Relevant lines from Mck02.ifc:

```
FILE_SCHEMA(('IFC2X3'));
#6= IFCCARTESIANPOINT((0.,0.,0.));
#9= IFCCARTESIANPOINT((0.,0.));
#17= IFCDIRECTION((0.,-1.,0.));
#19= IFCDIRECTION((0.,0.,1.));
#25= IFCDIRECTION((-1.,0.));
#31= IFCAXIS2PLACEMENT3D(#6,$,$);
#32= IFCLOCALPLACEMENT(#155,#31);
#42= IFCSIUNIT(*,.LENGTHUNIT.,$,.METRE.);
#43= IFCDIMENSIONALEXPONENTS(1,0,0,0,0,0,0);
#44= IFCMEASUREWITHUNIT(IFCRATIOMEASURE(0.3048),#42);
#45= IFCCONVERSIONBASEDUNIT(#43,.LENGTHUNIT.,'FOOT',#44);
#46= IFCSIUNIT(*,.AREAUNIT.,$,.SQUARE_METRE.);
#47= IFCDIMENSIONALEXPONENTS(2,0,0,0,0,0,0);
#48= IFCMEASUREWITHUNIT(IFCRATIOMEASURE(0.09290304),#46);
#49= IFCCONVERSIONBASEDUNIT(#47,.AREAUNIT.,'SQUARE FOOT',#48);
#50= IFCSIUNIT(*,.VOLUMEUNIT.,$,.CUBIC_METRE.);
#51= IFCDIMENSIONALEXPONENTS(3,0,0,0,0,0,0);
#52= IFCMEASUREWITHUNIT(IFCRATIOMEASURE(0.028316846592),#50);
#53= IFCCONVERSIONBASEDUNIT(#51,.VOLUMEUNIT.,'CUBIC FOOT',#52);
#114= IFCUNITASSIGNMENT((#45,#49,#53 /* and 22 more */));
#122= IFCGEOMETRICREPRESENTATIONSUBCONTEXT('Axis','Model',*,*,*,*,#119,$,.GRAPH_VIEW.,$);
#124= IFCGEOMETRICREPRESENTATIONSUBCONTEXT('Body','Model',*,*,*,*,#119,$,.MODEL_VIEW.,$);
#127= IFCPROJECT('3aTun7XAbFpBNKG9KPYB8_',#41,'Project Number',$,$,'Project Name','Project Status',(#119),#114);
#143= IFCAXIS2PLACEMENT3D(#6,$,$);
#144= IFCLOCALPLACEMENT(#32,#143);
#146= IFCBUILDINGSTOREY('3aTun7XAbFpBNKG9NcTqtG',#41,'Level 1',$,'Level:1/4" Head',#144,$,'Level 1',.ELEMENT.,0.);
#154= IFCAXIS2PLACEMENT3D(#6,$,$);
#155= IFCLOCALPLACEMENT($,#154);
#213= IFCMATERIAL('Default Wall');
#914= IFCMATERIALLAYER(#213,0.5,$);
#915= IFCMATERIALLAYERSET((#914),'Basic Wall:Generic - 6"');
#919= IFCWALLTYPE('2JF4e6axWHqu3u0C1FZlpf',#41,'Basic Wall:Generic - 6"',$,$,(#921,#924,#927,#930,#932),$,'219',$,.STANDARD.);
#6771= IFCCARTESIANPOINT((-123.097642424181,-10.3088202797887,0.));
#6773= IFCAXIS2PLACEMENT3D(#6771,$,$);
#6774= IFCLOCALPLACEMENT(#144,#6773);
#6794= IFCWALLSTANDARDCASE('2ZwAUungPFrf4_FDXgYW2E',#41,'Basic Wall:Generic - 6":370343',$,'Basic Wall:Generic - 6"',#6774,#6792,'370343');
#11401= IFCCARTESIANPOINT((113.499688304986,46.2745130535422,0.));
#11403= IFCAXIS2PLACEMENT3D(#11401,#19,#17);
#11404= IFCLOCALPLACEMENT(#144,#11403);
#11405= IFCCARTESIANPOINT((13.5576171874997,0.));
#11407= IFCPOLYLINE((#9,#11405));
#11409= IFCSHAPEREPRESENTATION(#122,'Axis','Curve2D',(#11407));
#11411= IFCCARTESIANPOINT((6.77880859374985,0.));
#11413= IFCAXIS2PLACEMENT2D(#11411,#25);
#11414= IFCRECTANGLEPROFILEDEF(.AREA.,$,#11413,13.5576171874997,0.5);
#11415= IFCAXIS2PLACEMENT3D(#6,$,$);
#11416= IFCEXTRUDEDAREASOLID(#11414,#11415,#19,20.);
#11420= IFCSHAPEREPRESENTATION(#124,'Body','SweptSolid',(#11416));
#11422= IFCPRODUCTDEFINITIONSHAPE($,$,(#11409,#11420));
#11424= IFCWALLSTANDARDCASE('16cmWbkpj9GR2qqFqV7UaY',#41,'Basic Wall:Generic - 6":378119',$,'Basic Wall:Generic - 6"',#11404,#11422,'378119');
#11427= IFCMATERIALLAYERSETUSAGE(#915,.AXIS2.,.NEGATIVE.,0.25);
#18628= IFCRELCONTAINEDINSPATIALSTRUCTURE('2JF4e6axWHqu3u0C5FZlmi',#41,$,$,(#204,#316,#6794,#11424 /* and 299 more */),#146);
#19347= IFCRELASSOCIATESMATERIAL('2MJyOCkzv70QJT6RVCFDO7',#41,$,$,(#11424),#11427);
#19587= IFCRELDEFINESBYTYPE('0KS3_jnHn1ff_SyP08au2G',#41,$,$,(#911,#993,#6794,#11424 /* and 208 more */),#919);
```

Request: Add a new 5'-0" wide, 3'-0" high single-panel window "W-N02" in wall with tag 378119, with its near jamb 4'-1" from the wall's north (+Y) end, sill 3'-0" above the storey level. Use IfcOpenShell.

```python
import numpy as np
import ifcopenshell
import ifcopenshell.api.feature
import ifcopenshell.api.geometry
import ifcopenshell.api.root
import ifcopenshell.api.spatial
import ifcopenshell.api.type
import ifcopenshell.geom
import ifcopenshell.util.element
import ifcopenshell.util.placement
import ifcopenshell.util.representation
import ifcopenshell.util.shape
import ifcopenshell.util.unit

model = ifcopenshell.open("Mck02.ifc")
unit_scale = ifcopenshell.util.unit.calculate_unit_scale(model)
settings = ifcopenshell.geom.settings()


def volume(element):
    """Net volume in cubic metres, openings subtracted."""
    shape = ifcopenshell.geom.create_shape(settings, element)
    return ifcopenshell.util.shape.get_volume(shape.geometry)


wall = model.by_guid("16cmWbkpj9GR2qqFqV7UaY")
storey = ifcopenshell.util.element.get_container(wall, ifc_class="IfcBuildingStorey")
context = ifcopenshell.util.representation.get_context(model, "Model", "Body", "MODEL_VIEW")
before = volume(wall)

width, height, from_end, sill = 1.524, 0.9144, 1.2446, 0.9144  # metres

# The wall runs along its own X axis, and the end named is its -X end.
wall_shape = ifcopenshell.geom.create_shape(settings, wall)
x, y, z = ifcopenshell.util.shape.get_vertices(wall_shape.geometry).T
start = x.min() + from_end
face, thickness = float(y.min()), float(y.max() - y.min())
wall_matrix = ifcopenshell.util.placement.get_local_placement(wall.ObjectPlacement)
level = ifcopenshell.util.placement.get_local_placement(storey.ObjectPlacement)[2, 3]


def in_wall(x, y):
    """Placement at x, y metres in the wall's axes, at sill height."""
    matrix = wall_matrix.copy()
    matrix[:, 3] = wall_matrix @ np.array([x / unit_scale, y / unit_scale, 0.0, 1.0])
    matrix[2, 3] = level + sill / unit_scale
    return matrix


# Opening: a box that overshoots both wall faces by 50 mm.
opening = ifcopenshell.api.root.create_entity(model, ifc_class="IfcOpeningElement")
box = ifcopenshell.api.geometry.add_wall_representation(
    model, context=context, length=width, height=height, thickness=thickness + 0.1
)
ifcopenshell.api.geometry.assign_representation(model, product=opening, representation=box)
ifcopenshell.api.geometry.edit_object_placement(model, product=opening, matrix=in_wall(start, face - 0.05), is_si=False)
ifcopenshell.api.feature.add_feature(model, feature=opening, element=wall)

window = ifcopenshell.api.root.create_entity(model, ifc_class="IfcWindow", name="W-N02")
window.OverallWidth, window.OverallHeight = width / unit_scale, height / unit_scale
body = ifcopenshell.api.geometry.add_window_representation(
    model,
    context=context,
    overall_width=window.OverallWidth,
    overall_height=window.OverallHeight,
    partition_type="SINGLE_PANEL",
)
ifcopenshell.api.geometry.assign_representation(model, product=window, representation=body)
ifcopenshell.api.spatial.assign_container(model, products=[window], relating_structure=storey)
fills = ifcopenshell.api.feature.add_filling(model, opening=opening, element=window)
fills.OwnerHistory = window.OwnerHistory  # required in IFC2X3

# IFC2X3 keeps the operation on the window style.
style = ifcopenshell.api.root.create_entity(model, ifc_class="IfcWindowStyle", name="W-N02")
style.OperationType, style.ConstructionType = "SINGLE_PANEL", "NOTDEFINED"
style.ParameterTakesPrecedence = style.Sizeable = False
ifcopenshell.api.type.assign_type(model, related_objects=[window], relating_type=style)

# Centre the window in the wall's thickness.
ifcopenshell.api.geometry.edit_object_placement(model, product=window, matrix=in_wall(start, face), is_si=False)
window_shape = ifcopenshell.geom.create_shape(settings, window)
depth = ifcopenshell.util.shape.get_vertices(window_shape.geometry)[:, 1]
offset = face + thickness / 2 - (depth.min() + depth.max()) / 2
ifcopenshell.api.geometry.edit_object_placement(model, product=window, matrix=in_wall(start, offset), is_si=False)

after = volume(wall)

print(f"wall volume {before:.3f} -> {after:.3f} m3")

model.write("Mck02_v2.ifc")
```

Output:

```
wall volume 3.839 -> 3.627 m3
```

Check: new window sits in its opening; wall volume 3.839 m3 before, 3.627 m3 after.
